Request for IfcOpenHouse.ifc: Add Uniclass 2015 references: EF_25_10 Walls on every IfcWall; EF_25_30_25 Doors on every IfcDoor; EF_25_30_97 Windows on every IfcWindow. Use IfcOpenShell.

First a look at what the model holds.

```python
import ifcopenshell

model = ifcopenshell.open("IfcOpenHouse.ifc")
print(model.schema)
print("classifications:", [c.Name for c in model.by_type("IfcClassification")])
for ifc_class in ("IfcDoor", "IfcRoof", "IfcStair", "IfcWall", "IfcWindow"):
    print(ifc_class, len(model.by_type(ifc_class)))
```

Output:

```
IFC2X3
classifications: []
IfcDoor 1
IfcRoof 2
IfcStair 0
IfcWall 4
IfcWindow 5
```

```python
import ifcopenshell
import ifcopenshell.api.classification

model = ifcopenshell.open("IfcOpenHouse.ifc")

# IFC2X3 requires Source and Edition and has no link from the project to the system.
system = model.create_entity("IfcClassification", Source="NBS", Edition="2015", Name="Uniclass 2015")

codes = {
    "IfcWall": ("EF_25_10", "Walls"),
    "IfcDoor": ("EF_25_30_25", "Doors"),
    "IfcWindow": ("EF_25_30_97", "Windows"),
}
for ifc_class, (code, name) in codes.items():
    products = model.by_type(ifc_class)
    ifcopenshell.api.classification.add_reference(
        model, products=products, classification=system, identification=code, name=name
    )
    print(code, len(products))

model.write("IfcOpenHouse_rev.ifc")
```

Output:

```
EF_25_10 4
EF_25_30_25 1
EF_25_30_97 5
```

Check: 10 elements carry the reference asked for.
